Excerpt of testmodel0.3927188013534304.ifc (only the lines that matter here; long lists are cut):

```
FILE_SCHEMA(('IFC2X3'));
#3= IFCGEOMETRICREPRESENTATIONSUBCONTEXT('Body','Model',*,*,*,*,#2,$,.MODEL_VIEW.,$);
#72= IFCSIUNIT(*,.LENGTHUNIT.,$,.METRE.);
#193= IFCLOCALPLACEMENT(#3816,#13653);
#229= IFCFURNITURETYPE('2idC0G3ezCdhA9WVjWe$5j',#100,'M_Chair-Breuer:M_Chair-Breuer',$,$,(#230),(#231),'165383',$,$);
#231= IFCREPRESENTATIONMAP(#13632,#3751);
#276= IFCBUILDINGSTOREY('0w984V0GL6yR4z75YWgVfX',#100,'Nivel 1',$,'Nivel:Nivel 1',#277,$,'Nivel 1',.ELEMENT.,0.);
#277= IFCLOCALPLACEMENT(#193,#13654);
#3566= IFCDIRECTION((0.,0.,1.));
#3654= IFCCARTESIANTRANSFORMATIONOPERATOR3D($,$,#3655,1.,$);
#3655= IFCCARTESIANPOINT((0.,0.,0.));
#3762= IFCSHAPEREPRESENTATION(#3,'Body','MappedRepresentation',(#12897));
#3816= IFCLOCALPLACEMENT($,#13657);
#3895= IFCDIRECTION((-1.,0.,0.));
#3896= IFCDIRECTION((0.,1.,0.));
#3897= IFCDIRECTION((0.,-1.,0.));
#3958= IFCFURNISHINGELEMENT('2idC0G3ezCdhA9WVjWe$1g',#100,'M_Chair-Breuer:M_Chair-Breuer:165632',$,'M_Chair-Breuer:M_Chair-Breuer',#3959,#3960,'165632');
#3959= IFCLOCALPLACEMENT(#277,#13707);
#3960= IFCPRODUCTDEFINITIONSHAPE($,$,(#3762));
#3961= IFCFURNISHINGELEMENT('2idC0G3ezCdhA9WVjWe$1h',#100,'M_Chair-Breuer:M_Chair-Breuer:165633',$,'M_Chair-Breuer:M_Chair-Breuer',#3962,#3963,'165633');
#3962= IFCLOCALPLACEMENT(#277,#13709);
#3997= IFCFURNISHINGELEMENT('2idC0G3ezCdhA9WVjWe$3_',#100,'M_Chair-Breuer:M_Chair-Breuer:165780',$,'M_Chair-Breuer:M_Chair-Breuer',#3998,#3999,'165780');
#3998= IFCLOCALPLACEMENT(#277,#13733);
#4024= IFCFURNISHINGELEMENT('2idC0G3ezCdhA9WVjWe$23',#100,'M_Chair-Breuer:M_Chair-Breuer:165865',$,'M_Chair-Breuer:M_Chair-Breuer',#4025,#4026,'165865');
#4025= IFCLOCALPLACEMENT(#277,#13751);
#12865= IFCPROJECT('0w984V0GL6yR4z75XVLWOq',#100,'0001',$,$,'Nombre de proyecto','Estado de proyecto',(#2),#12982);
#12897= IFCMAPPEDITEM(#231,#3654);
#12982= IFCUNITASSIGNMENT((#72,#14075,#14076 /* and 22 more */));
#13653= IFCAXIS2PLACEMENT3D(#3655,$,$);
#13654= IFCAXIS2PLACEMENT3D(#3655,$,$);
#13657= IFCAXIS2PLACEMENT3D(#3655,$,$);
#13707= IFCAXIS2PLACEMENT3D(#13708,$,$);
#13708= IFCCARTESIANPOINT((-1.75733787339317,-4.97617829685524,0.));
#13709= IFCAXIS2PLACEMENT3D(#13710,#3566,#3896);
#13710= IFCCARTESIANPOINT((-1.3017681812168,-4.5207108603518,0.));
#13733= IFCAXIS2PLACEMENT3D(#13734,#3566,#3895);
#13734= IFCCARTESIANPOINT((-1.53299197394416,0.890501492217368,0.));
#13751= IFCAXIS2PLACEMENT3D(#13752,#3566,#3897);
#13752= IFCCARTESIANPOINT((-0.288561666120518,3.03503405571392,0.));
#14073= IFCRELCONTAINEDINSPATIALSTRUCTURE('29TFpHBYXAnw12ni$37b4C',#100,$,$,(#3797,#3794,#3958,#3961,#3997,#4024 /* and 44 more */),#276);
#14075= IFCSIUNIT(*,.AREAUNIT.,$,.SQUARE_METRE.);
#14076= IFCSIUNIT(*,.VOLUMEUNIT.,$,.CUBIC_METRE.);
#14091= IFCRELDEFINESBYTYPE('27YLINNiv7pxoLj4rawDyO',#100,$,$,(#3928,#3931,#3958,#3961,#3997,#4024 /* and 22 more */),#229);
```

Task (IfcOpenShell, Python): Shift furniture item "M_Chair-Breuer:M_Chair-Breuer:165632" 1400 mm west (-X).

```python
import ifcopenshell
import ifcopenshell.api.geometry
import ifcopenshell.util.placement
import ifcopenshell.util.unit

model = ifcopenshell.open("testmodel0.3927188013534304.ifc")
unit_scale = ifcopenshell.util.unit.calculate_unit_scale(model)

item = model.by_guid("2idC0G3ezCdhA9WVjWe$1g")
matrix = ifcopenshell.util.placement.get_local_placement(item.ObjectPlacement)
matrix[0, 3] -= 1.4 / unit_scale
ifcopenshell.api.geometry.edit_object_placement(model, product=item, matrix=matrix, is_si=False)

print(ifcopenshell.util.placement.get_local_placement(item.ObjectPlacement).round(3) + 0.0)

model.write("testmodel0.3927188013534304_edited.ifc")
```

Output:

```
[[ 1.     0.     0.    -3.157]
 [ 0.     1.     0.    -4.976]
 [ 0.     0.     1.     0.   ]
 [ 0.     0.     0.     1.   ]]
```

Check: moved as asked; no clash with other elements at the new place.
